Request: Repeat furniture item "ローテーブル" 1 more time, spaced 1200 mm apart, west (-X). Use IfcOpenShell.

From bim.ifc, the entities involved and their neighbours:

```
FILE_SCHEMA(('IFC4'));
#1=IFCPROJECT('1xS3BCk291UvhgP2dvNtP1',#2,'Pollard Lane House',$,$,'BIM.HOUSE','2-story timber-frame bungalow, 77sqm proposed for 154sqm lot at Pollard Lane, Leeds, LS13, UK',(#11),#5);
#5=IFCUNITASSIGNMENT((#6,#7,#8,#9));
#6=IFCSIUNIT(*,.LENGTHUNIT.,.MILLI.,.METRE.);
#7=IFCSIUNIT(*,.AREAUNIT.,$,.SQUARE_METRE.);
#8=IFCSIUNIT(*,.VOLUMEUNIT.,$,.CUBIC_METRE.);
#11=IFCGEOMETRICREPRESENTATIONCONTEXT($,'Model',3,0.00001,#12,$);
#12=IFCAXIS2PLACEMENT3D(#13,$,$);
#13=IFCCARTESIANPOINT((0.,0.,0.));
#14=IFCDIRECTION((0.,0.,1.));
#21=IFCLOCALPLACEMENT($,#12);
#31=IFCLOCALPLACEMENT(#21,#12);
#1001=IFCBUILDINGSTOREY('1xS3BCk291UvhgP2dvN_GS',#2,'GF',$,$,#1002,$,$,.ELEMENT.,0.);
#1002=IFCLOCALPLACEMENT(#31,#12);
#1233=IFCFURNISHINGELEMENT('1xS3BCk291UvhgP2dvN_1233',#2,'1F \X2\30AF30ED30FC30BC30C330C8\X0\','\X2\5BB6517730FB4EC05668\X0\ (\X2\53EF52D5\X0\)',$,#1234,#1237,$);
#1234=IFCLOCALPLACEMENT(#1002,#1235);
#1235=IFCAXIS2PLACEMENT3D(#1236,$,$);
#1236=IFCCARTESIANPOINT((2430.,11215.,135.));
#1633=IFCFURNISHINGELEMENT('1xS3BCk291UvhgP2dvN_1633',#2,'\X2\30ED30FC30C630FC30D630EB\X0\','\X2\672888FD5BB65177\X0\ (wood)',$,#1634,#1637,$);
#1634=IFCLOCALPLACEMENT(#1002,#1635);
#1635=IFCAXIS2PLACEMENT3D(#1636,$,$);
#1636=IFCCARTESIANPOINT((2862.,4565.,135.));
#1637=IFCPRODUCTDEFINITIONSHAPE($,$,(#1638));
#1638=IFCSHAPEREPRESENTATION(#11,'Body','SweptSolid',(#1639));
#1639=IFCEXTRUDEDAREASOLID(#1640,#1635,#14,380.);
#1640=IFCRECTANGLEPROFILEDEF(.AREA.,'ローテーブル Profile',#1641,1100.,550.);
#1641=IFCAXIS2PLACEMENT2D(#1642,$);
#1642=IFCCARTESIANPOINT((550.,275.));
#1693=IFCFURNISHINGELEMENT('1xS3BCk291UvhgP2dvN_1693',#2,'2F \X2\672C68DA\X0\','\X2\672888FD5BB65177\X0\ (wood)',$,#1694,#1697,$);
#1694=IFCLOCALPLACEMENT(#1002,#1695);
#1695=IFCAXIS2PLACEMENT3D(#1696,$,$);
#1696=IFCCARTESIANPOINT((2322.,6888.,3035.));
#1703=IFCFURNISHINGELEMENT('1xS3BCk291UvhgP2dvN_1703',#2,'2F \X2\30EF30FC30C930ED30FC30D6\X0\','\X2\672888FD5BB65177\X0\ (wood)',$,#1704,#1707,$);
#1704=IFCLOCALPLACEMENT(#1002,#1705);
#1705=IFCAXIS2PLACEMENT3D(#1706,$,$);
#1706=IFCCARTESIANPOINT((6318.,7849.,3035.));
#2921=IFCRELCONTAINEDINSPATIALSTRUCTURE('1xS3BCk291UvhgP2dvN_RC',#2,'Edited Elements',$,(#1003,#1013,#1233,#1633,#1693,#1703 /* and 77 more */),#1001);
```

```python
import numpy as np
import ifcopenshell
import ifcopenshell.api.geometry
import ifcopenshell.api.root
import ifcopenshell.util.element
import ifcopenshell.util.placement

model = ifcopenshell.open("bim.ifc")


def reuse_history(source, copy):
    """copy_class also copies each property set's owner history, people and application; keep the originals."""
    for rel in copy.IsDefinedBy:
        if rel.is_a("IfcRelDefinesByProperties") and (history := rel.RelatingPropertyDefinition.OwnerHistory):
            rel.RelatingPropertyDefinition.OwnerHistory = source.OwnerHistory
            ifcopenshell.util.element.remove_deep2(model, history)


source = model.by_id(1633)
base = ifcopenshell.util.placement.get_local_placement(source.ObjectPlacement)
step = np.array([-1.0, 0.0, 0.0]) * 1200.0

for i in range(1, 2):
    copy = ifcopenshell.api.root.copy_class(model, product=source)
    copy.Representation = ifcopenshell.util.element.copy_deep(
        model, source.Representation, exclude=["IfcGeometricRepresentationContext", "IfcRepresentationMap"]
    )
    reuse_history(source, copy)
    matrix = base.copy()
    matrix[:3, 3] += i * step
    print("added at", matrix[:3, 3].round(3) + 0.0)
    ifcopenshell.api.geometry.edit_object_placement(model, product=copy, matrix=matrix, is_si=False)

model.write("bim-out.ifc")
```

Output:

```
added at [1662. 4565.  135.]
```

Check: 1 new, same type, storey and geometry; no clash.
